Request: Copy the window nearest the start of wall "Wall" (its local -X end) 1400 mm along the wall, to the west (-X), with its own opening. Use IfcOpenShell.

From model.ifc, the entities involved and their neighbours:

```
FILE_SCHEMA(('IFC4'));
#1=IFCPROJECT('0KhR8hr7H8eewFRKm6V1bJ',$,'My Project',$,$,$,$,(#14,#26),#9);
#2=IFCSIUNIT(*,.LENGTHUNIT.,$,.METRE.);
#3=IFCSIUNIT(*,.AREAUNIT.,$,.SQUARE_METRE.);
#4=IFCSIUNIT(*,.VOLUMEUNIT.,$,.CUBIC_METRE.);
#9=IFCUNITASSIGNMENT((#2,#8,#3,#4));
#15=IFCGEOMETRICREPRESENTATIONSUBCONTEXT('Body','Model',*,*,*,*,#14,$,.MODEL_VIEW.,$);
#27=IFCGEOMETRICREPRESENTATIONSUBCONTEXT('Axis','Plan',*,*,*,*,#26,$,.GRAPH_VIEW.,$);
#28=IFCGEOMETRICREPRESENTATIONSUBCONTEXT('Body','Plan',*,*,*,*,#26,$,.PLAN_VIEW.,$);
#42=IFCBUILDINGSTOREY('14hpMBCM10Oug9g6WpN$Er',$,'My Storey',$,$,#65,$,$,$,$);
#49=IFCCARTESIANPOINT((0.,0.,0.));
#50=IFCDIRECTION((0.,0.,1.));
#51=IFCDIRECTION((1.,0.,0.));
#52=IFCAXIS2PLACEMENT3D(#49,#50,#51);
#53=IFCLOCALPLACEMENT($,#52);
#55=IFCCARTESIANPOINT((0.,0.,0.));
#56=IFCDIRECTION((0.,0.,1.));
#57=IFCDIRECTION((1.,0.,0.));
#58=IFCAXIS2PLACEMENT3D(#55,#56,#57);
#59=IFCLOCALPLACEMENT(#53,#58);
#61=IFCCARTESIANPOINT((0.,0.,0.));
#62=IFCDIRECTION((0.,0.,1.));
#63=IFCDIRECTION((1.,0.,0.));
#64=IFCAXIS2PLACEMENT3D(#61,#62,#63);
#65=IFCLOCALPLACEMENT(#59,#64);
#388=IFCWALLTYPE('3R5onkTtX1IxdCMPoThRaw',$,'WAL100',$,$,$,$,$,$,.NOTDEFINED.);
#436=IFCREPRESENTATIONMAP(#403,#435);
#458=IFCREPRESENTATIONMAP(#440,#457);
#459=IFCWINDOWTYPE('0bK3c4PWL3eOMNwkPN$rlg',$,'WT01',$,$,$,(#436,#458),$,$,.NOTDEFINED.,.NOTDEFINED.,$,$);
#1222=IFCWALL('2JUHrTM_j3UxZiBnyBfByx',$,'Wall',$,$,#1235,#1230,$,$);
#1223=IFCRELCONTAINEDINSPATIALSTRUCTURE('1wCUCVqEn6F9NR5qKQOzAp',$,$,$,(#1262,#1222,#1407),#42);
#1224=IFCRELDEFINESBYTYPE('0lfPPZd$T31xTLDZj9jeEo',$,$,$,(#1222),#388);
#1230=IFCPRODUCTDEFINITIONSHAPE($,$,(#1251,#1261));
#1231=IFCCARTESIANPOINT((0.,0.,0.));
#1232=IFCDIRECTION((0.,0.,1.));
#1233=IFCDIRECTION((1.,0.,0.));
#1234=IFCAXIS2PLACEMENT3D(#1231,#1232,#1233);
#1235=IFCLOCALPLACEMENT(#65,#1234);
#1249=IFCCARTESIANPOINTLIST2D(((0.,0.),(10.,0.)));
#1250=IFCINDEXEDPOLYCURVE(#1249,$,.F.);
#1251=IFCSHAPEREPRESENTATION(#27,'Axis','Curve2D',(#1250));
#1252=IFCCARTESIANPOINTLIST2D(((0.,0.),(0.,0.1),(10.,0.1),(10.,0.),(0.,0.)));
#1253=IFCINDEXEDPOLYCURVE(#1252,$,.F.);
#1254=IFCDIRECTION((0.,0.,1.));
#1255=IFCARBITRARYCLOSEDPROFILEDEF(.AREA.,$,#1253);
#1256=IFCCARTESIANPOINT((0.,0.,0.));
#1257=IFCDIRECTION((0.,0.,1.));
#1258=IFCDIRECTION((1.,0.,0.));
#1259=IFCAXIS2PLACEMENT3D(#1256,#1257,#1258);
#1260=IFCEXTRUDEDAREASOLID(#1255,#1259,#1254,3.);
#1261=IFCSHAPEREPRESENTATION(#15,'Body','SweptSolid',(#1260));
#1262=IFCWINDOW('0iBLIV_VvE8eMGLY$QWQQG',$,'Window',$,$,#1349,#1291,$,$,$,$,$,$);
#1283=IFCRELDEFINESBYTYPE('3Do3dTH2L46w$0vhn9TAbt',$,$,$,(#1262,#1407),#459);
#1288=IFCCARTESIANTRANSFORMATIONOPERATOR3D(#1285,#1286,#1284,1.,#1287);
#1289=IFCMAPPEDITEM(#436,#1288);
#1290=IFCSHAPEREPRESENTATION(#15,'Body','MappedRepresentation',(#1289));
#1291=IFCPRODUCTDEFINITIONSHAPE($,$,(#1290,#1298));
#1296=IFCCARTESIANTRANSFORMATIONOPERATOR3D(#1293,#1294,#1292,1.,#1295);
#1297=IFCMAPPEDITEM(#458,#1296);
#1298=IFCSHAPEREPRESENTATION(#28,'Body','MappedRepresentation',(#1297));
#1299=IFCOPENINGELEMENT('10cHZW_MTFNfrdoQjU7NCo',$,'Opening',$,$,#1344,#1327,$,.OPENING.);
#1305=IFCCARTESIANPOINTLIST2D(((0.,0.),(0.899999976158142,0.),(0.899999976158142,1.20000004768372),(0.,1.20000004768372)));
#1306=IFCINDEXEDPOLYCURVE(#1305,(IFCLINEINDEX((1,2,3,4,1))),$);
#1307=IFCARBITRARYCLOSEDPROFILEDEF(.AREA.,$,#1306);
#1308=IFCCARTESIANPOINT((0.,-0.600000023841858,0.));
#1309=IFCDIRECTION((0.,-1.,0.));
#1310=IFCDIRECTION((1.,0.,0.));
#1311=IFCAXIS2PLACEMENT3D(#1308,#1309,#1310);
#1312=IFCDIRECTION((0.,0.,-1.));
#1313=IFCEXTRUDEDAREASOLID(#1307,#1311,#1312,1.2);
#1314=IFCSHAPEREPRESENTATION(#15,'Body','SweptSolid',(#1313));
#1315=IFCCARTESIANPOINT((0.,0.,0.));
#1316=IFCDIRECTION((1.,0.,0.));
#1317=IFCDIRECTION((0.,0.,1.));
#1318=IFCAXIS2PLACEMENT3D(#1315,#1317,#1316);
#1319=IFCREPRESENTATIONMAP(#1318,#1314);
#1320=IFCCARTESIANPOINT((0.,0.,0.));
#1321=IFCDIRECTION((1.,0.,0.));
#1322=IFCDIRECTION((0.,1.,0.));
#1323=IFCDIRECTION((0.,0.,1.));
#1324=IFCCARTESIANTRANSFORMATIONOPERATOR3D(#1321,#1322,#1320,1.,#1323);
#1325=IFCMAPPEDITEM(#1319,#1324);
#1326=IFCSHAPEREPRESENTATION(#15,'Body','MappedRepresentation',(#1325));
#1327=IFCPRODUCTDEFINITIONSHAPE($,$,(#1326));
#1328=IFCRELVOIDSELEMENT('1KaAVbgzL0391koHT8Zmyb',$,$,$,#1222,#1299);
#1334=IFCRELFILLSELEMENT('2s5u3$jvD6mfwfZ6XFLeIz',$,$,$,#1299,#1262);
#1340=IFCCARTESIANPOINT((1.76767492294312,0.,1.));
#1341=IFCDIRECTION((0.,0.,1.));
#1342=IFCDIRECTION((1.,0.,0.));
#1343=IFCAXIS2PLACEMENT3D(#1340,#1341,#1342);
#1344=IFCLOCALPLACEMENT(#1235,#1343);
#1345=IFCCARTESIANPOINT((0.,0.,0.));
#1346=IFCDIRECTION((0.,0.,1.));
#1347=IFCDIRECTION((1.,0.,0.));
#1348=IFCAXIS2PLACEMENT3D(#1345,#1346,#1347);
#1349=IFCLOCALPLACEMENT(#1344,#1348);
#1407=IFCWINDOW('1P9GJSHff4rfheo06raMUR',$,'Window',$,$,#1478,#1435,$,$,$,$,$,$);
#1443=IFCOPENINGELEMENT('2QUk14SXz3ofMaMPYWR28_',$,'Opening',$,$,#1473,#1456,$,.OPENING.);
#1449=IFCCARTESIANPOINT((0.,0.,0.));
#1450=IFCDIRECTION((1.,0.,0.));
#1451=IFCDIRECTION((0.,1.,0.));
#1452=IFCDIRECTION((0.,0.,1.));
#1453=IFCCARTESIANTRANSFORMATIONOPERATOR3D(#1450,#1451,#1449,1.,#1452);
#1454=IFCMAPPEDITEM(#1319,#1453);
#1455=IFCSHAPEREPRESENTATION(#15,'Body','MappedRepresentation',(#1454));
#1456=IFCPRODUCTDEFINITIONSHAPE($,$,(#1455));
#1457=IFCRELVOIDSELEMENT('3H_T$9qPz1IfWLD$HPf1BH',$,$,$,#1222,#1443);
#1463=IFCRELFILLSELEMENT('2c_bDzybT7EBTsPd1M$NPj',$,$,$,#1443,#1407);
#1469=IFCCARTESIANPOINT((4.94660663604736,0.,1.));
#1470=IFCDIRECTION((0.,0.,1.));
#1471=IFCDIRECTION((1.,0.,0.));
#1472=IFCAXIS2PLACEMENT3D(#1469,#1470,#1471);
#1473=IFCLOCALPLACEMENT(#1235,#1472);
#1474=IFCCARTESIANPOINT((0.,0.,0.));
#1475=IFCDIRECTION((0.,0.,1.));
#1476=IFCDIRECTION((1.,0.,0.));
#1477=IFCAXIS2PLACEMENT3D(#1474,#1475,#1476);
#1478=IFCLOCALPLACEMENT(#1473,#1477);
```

```python
import ifcopenshell
import ifcopenshell.api.feature
import ifcopenshell.api.geometry
import ifcopenshell.api.root
import ifcopenshell.geom
import ifcopenshell.util.element
import ifcopenshell.util.placement
import ifcopenshell.util.shape
import ifcopenshell.util.unit

model = ifcopenshell.open("model.ifc")
unit_scale = ifcopenshell.util.unit.calculate_unit_scale(model)
settings = ifcopenshell.geom.settings()


def volume(element):
    """Net volume in cubic metres, openings subtracted."""
    shape = ifcopenshell.geom.create_shape(settings, element)
    return ifcopenshell.util.shape.get_volume(shape.geometry)


window = model.by_id(1262)
opening = window.FillsVoids[0].RelatingOpeningElement
wall = opening.VoidsElements[0].RelatingBuildingElement
before = volume(wall)
shift = ifcopenshell.util.placement.get_local_placement(wall.ObjectPlacement)[:3, 0] * -1.4 / unit_scale

# copy_class copies the void relationship, type, container and properties, but no geometry.
new_opening = ifcopenshell.api.root.copy_class(model, product=opening)
new_opening.Representation = ifcopenshell.util.element.copy_deep(
    model, opening.Representation, exclude=["IfcGeometricRepresentationContext", "IfcRepresentationMap"]
)
new_window = ifcopenshell.api.root.copy_class(model, product=window)
new_window.Representation = ifcopenshell.util.element.copy_deep(
    model, window.Representation, exclude=["IfcGeometricRepresentationContext", "IfcRepresentationMap"]
)
ifcopenshell.api.feature.add_filling(model, opening=new_opening, element=new_window)

for old, new in ((opening, new_opening), (window, new_window)):
    matrix = ifcopenshell.util.placement.get_local_placement(old.ObjectPlacement)
    matrix[:3, 3] += shift
    ifcopenshell.api.geometry.edit_object_placement(model, product=new, matrix=matrix, is_si=False)

after = volume(wall)

print(f"wall volume {before:.3f} -> {after:.3f} m3")

model.write("model_edited.ifc")
```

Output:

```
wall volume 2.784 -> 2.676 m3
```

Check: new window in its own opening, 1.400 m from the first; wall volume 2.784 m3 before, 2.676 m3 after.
